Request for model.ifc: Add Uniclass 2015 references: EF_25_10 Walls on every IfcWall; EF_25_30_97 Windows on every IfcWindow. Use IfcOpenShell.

First a look at what the model holds.

```python
import ifcopenshell

model = ifcopenshell.open("model.ifc")
print(model.schema)
print("classifications:", [c.Name for c in model.by_type("IfcClassification")])
for ifc_class in ("IfcDoor", "IfcRoof", "IfcStair", "IfcWall", "IfcWindow"):
    print(ifc_class, len(model.by_type(ifc_class)))
```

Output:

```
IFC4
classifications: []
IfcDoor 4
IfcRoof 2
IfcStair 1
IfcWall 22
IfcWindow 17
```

```python
import ifcopenshell
import ifcopenshell.api.classification

model = ifcopenshell.open("model.ifc")

system = ifcopenshell.api.classification.add_classification(model, classification="Uniclass 2015")

codes = {
    "IfcWall": ("EF_25_10", "Walls"),
    "IfcWindow": ("EF_25_30_97", "Windows"),
}
for ifc_class, (code, name) in codes.items():
    products = model.by_type(ifc_class)
    ifcopenshell.api.classification.add_reference(
        model, products=products, classification=system, identification=code, name=name
    )
    print(code, len(products))

model.write("model_v2.ifc")
```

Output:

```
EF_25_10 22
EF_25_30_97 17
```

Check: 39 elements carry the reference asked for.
